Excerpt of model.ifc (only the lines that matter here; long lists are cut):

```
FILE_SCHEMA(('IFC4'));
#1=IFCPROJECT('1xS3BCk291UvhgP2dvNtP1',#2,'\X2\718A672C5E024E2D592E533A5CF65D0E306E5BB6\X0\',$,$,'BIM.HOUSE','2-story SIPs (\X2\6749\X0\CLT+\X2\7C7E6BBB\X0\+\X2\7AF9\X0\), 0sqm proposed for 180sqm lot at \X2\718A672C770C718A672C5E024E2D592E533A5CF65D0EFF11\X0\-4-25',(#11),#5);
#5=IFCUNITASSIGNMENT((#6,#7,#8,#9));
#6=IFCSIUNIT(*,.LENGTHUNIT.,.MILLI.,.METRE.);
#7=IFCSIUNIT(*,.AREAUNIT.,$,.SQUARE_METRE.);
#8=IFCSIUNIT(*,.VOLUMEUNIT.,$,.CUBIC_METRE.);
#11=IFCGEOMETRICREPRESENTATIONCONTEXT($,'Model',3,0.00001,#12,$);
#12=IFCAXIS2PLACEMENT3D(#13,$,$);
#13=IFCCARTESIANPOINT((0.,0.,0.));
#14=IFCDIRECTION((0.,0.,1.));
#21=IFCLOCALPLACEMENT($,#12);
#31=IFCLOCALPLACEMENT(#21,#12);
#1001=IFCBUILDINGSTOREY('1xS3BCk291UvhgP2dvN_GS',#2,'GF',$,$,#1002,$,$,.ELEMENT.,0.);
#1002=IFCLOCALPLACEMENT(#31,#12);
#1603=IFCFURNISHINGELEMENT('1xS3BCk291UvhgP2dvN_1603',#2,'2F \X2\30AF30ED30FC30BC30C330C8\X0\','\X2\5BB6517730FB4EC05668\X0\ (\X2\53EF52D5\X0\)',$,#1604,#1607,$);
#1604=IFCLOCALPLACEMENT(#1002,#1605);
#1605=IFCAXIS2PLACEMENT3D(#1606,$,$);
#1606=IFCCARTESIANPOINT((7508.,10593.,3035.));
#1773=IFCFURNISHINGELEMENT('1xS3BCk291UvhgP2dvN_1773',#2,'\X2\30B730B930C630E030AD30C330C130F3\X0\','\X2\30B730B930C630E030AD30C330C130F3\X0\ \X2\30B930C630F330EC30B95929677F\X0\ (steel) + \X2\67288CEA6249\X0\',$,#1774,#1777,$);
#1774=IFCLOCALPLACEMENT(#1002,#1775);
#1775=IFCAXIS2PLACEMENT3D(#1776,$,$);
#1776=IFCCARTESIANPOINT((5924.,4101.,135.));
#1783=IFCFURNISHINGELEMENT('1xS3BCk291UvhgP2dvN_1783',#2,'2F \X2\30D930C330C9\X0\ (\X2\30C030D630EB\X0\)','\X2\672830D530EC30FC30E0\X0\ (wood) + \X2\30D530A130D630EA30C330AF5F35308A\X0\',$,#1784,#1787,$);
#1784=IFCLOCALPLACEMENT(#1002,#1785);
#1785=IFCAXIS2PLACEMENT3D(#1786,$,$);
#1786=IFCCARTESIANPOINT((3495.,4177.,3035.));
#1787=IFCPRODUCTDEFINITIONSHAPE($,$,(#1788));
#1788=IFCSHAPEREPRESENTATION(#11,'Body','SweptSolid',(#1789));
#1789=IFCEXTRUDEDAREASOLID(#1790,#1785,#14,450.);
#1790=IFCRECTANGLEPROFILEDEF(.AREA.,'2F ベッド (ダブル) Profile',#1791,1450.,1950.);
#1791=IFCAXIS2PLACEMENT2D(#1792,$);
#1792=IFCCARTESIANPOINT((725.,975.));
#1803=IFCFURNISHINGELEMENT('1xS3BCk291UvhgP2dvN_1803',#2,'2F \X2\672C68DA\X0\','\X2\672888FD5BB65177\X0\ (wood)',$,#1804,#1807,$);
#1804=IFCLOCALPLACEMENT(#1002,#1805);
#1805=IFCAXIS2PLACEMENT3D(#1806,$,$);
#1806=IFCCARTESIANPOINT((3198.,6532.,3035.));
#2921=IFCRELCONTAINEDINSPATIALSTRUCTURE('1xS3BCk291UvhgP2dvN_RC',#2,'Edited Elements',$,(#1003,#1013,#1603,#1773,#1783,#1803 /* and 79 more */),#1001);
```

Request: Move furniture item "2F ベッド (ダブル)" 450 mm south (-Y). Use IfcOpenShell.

```python
import ifcopenshell
import ifcopenshell.api.geometry
import ifcopenshell.util.placement
import ifcopenshell.util.unit

model = ifcopenshell.open("model.ifc")
unit_scale = ifcopenshell.util.unit.calculate_unit_scale(model)

item = model.by_guid("1xS3BCk291UvhgP2dvN_1783")
matrix = ifcopenshell.util.placement.get_local_placement(item.ObjectPlacement)
matrix[1, 3] -= 0.45 / unit_scale
ifcopenshell.api.geometry.edit_object_placement(model, product=item, matrix=matrix, is_si=False)

print(ifcopenshell.util.placement.get_local_placement(item.ObjectPlacement).round(3) + 0.0)

model.write("model-out.ifc")
```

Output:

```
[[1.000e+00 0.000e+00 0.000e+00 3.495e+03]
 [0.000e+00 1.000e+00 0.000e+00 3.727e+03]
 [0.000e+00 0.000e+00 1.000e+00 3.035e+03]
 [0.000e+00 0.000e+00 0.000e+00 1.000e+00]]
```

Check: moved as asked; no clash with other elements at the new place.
